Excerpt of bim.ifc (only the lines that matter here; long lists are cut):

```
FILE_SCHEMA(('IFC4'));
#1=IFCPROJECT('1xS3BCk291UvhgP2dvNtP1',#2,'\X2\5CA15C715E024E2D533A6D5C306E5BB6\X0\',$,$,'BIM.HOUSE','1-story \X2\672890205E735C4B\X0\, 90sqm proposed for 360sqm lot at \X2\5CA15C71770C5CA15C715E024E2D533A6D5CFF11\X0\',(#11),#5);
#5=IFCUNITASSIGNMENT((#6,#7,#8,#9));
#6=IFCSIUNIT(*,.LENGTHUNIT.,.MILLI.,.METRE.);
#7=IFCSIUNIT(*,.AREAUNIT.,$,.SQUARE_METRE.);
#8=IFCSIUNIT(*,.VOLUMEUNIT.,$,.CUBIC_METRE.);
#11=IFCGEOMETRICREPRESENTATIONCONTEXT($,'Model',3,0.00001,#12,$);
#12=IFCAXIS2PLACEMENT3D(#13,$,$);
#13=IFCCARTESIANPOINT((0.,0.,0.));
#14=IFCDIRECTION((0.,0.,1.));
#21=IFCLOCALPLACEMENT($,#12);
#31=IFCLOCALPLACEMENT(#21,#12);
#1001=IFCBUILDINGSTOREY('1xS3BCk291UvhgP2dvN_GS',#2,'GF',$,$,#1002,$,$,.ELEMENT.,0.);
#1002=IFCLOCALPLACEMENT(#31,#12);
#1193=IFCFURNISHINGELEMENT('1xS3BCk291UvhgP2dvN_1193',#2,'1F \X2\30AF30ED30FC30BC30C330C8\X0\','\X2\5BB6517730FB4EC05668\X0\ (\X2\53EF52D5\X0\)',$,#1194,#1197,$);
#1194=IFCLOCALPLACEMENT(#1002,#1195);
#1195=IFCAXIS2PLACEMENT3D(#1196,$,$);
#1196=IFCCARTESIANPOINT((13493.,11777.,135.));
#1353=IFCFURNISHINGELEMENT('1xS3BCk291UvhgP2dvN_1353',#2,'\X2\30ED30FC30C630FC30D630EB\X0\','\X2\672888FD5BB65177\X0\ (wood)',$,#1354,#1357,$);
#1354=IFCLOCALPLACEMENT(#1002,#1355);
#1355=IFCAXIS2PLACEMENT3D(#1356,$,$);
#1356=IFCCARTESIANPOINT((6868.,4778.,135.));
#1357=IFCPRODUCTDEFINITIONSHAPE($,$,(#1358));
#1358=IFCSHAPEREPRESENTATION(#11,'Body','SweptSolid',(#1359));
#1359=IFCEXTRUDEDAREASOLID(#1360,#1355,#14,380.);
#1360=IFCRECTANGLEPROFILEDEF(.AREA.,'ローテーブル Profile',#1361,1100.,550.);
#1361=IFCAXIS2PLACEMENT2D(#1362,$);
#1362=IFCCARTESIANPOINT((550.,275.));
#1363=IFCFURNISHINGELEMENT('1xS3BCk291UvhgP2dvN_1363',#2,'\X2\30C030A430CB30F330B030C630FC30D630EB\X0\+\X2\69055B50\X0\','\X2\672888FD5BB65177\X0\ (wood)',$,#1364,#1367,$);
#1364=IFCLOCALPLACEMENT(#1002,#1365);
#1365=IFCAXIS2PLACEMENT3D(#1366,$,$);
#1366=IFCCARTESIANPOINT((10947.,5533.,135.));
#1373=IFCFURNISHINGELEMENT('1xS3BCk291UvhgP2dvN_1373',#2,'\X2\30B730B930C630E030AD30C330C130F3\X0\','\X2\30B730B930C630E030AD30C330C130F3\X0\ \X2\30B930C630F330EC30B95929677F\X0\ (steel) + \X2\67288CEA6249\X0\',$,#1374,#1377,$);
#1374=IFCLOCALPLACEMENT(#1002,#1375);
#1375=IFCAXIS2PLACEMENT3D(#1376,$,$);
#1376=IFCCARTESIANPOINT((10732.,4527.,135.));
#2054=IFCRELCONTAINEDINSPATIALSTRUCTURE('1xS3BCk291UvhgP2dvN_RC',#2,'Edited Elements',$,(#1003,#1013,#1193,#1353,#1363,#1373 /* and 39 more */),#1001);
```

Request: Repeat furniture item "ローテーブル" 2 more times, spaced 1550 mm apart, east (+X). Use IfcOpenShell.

```python
import numpy as np
import ifcopenshell
import ifcopenshell.api.geometry
import ifcopenshell.api.root
import ifcopenshell.util.element
import ifcopenshell.util.placement

model = ifcopenshell.open("bim.ifc")


def reuse_history(source, copy):
    """copy_class also copies each property set's owner history, people and application; keep the originals."""
    for rel in copy.IsDefinedBy:
        if rel.is_a("IfcRelDefinesByProperties") and (history := rel.RelatingPropertyDefinition.OwnerHistory):
            rel.RelatingPropertyDefinition.OwnerHistory = source.OwnerHistory
            ifcopenshell.util.element.remove_deep2(model, history)


source = model.by_guid("1xS3BCk291UvhgP2dvN_1353")
base = ifcopenshell.util.placement.get_local_placement(source.ObjectPlacement)
step = np.array([1.0, 0.0, 0.0]) * 1550.0

for i in range(1, 3):
    copy = ifcopenshell.api.root.copy_class(model, product=source)
    copy.Representation = ifcopenshell.util.element.copy_deep(
        model, source.Representation, exclude=["IfcGeometricRepresentationContext", "IfcRepresentationMap"]
    )
    reuse_history(source, copy)
    matrix = base.copy()
    matrix[:3, 3] += i * step
    print("added at", matrix[:3, 3].round(3) + 0.0)
    ifcopenshell.api.geometry.edit_object_placement(model, product=copy, matrix=matrix, is_si=False)

model.write("bim-out.ifc")
```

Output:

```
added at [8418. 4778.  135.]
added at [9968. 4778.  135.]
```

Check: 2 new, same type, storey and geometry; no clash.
